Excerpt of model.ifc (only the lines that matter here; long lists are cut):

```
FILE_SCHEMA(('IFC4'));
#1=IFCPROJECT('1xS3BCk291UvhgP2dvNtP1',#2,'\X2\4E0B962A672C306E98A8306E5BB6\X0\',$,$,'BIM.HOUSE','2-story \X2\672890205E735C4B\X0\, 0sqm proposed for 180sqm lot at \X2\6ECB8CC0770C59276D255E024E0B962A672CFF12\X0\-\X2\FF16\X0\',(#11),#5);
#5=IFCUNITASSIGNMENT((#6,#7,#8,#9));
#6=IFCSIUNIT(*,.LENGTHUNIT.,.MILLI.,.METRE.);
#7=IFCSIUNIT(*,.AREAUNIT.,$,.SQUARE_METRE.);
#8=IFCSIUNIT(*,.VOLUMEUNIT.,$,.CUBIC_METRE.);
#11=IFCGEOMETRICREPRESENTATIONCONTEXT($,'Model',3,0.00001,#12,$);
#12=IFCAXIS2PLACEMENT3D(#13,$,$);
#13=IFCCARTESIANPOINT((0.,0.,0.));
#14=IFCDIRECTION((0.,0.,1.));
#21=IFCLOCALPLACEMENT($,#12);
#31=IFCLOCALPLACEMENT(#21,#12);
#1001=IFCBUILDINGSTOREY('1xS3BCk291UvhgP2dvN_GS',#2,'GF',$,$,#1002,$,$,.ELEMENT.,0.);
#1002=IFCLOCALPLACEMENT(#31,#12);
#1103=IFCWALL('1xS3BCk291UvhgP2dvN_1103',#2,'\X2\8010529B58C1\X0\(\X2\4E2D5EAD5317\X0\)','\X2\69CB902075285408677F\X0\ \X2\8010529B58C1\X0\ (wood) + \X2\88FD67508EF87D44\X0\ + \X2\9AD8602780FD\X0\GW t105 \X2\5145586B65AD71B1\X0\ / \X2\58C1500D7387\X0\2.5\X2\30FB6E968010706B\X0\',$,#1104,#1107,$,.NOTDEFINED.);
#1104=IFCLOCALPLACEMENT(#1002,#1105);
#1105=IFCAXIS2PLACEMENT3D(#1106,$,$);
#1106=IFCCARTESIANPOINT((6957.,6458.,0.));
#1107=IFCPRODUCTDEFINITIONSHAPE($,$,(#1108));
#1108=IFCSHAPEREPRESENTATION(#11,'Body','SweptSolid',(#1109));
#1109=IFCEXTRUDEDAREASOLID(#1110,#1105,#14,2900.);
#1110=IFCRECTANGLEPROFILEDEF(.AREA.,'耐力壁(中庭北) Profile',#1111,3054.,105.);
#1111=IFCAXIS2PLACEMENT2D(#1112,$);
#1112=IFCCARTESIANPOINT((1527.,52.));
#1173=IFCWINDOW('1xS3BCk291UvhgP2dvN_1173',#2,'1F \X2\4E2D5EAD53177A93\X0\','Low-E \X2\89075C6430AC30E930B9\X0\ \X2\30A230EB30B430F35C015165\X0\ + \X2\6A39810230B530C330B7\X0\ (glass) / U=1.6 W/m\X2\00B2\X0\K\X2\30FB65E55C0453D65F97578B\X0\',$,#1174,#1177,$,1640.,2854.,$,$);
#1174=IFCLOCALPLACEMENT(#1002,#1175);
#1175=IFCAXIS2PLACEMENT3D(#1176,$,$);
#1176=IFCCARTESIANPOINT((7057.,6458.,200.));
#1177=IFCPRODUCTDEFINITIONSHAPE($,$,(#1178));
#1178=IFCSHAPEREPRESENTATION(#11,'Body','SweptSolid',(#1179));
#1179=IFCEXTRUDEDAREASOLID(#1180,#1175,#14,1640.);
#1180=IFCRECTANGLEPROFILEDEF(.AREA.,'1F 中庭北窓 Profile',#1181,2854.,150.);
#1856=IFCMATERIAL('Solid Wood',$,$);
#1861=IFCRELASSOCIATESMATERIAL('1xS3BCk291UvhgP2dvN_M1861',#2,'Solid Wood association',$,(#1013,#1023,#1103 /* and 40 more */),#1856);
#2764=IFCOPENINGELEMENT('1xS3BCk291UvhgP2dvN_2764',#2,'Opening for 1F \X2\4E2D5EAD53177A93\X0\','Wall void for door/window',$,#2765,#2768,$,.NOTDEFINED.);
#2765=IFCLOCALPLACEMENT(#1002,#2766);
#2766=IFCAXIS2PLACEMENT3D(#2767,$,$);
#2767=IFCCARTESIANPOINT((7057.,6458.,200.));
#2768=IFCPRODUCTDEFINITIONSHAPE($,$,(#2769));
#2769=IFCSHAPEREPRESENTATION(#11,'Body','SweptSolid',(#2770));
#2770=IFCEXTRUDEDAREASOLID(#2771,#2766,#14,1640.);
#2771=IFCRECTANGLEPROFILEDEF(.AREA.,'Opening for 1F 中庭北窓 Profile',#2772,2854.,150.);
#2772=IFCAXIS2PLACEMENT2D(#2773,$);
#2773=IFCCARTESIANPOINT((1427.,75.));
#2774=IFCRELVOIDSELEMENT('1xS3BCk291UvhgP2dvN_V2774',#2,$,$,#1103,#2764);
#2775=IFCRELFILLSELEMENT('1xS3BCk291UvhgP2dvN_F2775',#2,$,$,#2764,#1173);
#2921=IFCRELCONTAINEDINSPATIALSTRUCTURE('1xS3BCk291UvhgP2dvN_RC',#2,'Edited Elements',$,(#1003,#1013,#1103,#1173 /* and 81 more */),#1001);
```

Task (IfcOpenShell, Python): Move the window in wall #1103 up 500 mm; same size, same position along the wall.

```python
import numpy as np
import ifcopenshell
import ifcopenshell.api.geometry
import ifcopenshell.util.placement
import ifcopenshell.util.unit

model = ifcopenshell.open("model.ifc")
unit_scale = ifcopenshell.util.unit.calculate_unit_scale(model)

window = model.by_id(1173)
opening = window.FillsVoids[0].RelatingOpeningElement
dz = 500.0

shift = np.array([0.0, 0.0, dz])
# The window is not placed relative to its opening, so move both.
for product in (opening, window):
    matrix = ifcopenshell.util.placement.get_local_placement(product.ObjectPlacement)
    matrix[:3, 3] += shift
    ifcopenshell.api.geometry.edit_object_placement(model, product=product, matrix=matrix, is_si=False)

print(f"moved by {dz * unit_scale:+.3f} m")

model.write("model_rev.ifc")
```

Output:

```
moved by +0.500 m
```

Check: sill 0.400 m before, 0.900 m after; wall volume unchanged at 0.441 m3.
